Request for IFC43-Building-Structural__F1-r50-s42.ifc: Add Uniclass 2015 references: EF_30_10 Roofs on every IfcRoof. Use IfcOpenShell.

First a look at what the model holds.

```python
import ifcopenshell

model = ifcopenshell.open("IFC43-Building-Structural__F1-r50-s42.ifc")
print(model.schema)
print("classifications:", [c.Name for c in model.by_type("IfcClassification")])
for ifc_class in ("IfcDoor", "IfcRoof", "IfcStair", "IfcWall", "IfcWindow"):
    print(ifc_class, len(model.by_type(ifc_class)))
```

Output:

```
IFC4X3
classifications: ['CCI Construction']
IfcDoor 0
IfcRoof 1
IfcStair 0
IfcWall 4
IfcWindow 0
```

```python
import ifcopenshell
import ifcopenshell.api.classification

model = ifcopenshell.open("IFC43-Building-Structural__F1-r50-s42.ifc")

system = ifcopenshell.api.classification.add_classification(model, classification="Uniclass 2015")

codes = {
    "IfcRoof": ("EF_30_10", "Roofs"),
}
for ifc_class, (code, name) in codes.items():
    products = model.by_type(ifc_class)
    ifcopenshell.api.classification.add_reference(
        model, products=products, classification=system, identification=code, name=name
    )
    print(code, len(products))

model.write("IFC43-Building-Structural__F1-r50-s42_edited.ifc")
```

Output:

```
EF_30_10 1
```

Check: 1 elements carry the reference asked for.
